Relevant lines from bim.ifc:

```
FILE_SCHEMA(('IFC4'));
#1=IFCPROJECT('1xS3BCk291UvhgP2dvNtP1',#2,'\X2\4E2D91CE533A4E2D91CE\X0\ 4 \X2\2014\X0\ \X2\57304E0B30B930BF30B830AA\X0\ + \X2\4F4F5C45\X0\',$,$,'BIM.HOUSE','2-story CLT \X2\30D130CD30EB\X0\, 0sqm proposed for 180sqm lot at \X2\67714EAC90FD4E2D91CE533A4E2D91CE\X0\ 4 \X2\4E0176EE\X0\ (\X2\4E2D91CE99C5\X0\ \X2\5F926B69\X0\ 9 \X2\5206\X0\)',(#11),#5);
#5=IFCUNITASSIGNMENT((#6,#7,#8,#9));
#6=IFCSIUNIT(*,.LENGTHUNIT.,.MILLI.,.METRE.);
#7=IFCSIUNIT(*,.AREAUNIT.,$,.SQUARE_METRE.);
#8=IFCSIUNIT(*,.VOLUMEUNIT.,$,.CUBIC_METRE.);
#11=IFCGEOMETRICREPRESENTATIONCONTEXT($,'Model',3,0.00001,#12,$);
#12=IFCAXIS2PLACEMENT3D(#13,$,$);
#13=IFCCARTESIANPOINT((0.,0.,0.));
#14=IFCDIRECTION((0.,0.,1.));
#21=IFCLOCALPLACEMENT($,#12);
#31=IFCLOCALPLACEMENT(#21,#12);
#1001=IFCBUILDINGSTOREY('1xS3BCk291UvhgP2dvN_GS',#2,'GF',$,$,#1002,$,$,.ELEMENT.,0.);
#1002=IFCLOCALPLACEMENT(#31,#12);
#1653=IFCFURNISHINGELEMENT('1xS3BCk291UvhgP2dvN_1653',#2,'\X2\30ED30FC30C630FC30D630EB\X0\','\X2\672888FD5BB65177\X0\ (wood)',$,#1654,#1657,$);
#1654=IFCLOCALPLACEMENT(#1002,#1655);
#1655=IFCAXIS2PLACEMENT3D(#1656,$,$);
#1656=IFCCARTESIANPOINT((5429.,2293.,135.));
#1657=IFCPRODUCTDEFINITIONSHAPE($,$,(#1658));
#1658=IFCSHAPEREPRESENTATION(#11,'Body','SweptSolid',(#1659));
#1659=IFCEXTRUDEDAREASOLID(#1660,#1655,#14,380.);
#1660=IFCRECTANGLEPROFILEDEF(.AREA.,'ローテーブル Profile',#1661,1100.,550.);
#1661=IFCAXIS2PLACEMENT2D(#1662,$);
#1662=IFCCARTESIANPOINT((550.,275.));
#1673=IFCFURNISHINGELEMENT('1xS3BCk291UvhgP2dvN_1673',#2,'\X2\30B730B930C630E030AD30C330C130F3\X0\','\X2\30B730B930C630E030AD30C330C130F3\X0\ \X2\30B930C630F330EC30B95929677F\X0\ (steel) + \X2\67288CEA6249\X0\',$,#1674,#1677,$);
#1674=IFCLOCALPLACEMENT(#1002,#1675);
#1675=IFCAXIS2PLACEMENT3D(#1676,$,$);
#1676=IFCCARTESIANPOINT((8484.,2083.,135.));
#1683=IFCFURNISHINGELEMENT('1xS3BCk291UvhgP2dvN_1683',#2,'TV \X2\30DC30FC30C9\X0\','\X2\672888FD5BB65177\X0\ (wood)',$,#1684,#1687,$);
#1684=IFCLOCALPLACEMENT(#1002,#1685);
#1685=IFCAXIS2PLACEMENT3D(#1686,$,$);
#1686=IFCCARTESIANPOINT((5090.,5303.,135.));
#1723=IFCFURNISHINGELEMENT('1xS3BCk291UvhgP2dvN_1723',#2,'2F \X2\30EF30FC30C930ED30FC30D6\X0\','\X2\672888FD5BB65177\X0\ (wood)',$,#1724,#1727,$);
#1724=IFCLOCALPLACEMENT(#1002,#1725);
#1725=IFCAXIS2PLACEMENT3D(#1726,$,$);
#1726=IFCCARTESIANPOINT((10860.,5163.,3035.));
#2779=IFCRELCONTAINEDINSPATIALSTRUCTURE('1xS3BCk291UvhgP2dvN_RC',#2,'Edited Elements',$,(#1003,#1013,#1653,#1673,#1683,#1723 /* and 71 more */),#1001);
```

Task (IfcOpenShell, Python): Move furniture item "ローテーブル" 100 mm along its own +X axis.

```python
import ifcopenshell
import ifcopenshell.api.geometry
import ifcopenshell.util.placement

model = ifcopenshell.open("bim.ifc")

item = model.by_id(1653)
matrix = ifcopenshell.util.placement.get_local_placement(item.ObjectPlacement)
matrix[:3, 3] += matrix[:3, 0] * 100.0
ifcopenshell.api.geometry.edit_object_placement(model, product=item, matrix=matrix, is_si=False)

print(ifcopenshell.util.placement.get_local_placement(item.ObjectPlacement).round(3) + 0.0)

model.write("bim_edited.ifc")
```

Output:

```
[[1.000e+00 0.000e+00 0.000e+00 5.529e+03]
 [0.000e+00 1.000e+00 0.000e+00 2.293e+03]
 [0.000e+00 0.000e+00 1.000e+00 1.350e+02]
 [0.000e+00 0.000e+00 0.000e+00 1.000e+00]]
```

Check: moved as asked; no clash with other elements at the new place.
